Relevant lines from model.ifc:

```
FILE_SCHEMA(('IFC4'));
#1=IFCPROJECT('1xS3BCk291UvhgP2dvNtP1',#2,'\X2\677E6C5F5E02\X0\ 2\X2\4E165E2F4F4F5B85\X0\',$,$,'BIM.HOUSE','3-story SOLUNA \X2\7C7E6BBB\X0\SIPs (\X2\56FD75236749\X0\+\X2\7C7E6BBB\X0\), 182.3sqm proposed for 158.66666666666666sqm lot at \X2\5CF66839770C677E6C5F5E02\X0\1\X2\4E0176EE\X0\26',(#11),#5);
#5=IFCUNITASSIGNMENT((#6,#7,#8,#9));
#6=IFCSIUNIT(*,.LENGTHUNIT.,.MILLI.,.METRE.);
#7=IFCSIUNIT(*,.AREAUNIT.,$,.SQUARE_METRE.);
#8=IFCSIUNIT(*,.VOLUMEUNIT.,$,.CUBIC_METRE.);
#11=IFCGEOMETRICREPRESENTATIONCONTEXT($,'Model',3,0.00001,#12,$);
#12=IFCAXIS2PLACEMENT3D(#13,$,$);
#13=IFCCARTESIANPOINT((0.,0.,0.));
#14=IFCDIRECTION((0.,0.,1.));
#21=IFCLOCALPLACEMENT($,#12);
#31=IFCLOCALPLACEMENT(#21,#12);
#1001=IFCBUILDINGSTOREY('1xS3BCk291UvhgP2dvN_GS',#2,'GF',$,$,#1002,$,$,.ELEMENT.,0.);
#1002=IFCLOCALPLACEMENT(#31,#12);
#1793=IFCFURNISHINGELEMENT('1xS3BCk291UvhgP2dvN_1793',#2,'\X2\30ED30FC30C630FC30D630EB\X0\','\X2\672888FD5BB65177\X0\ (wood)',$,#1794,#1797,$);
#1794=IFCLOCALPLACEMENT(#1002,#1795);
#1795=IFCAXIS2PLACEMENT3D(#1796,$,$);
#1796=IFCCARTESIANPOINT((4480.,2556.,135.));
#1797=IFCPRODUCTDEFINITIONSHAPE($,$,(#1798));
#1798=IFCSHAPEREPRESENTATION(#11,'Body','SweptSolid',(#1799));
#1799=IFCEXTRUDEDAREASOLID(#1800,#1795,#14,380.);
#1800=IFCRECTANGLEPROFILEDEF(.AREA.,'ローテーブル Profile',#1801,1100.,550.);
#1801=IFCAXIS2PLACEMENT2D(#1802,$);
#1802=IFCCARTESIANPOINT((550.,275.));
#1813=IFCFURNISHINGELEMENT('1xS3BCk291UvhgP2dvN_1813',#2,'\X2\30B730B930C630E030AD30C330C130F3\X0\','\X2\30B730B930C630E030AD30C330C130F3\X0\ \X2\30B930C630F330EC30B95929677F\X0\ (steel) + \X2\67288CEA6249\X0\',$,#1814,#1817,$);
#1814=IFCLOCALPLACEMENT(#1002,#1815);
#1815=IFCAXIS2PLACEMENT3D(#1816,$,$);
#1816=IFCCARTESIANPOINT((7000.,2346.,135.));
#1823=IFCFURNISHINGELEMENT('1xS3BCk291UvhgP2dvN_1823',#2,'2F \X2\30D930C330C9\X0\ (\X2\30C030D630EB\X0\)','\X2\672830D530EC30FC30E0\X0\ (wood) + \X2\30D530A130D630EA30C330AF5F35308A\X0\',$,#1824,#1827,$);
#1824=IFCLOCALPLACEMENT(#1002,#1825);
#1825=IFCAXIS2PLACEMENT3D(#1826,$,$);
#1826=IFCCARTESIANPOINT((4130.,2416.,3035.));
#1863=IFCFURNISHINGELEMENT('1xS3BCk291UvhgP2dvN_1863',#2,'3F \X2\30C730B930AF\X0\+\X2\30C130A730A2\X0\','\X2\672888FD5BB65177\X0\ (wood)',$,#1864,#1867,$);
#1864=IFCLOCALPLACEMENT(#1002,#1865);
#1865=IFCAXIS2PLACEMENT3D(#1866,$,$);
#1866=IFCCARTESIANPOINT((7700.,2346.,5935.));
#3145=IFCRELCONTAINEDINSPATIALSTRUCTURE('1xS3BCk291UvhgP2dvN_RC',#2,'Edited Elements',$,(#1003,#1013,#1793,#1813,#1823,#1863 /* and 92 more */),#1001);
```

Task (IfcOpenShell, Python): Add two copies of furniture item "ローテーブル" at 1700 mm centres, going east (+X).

```python
import numpy as np
import ifcopenshell
import ifcopenshell.api.geometry
import ifcopenshell.api.root
import ifcopenshell.util.element
import ifcopenshell.util.placement
import ifcopenshell.util.unit

model = ifcopenshell.open("model.ifc")
unit_scale = ifcopenshell.util.unit.calculate_unit_scale(model)


def reuse_history(source, copy):
    """copy_class also copies each property set's owner history, people and application; keep the originals."""
    for rel in copy.IsDefinedBy:
        if rel.is_a("IfcRelDefinesByProperties") and (history := rel.RelatingPropertyDefinition.OwnerHistory):
            rel.RelatingPropertyDefinition.OwnerHistory = source.OwnerHistory
            ifcopenshell.util.element.remove_deep2(model, history)


source = model.by_guid("1xS3BCk291UvhgP2dvN_1793")
base = ifcopenshell.util.placement.get_local_placement(source.ObjectPlacement)
step = np.array([1.0, 0.0, 0.0]) * 1.7 / unit_scale

for i in range(1, 3):
    copy = ifcopenshell.api.root.copy_class(model, product=source)
    copy.Representation = ifcopenshell.util.element.copy_deep(
        model, source.Representation, exclude=["IfcGeometricRepresentationContext", "IfcRepresentationMap"]
    )
    reuse_history(source, copy)
    matrix = base.copy()
    matrix[:3, 3] += i * step
    print("added at", matrix[:3, 3].round(3) + 0.0)
    ifcopenshell.api.geometry.edit_object_placement(model, product=copy, matrix=matrix, is_si=False)

model.write("model-out.ifc")
```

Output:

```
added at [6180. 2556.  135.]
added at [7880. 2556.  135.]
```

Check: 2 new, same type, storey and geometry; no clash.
